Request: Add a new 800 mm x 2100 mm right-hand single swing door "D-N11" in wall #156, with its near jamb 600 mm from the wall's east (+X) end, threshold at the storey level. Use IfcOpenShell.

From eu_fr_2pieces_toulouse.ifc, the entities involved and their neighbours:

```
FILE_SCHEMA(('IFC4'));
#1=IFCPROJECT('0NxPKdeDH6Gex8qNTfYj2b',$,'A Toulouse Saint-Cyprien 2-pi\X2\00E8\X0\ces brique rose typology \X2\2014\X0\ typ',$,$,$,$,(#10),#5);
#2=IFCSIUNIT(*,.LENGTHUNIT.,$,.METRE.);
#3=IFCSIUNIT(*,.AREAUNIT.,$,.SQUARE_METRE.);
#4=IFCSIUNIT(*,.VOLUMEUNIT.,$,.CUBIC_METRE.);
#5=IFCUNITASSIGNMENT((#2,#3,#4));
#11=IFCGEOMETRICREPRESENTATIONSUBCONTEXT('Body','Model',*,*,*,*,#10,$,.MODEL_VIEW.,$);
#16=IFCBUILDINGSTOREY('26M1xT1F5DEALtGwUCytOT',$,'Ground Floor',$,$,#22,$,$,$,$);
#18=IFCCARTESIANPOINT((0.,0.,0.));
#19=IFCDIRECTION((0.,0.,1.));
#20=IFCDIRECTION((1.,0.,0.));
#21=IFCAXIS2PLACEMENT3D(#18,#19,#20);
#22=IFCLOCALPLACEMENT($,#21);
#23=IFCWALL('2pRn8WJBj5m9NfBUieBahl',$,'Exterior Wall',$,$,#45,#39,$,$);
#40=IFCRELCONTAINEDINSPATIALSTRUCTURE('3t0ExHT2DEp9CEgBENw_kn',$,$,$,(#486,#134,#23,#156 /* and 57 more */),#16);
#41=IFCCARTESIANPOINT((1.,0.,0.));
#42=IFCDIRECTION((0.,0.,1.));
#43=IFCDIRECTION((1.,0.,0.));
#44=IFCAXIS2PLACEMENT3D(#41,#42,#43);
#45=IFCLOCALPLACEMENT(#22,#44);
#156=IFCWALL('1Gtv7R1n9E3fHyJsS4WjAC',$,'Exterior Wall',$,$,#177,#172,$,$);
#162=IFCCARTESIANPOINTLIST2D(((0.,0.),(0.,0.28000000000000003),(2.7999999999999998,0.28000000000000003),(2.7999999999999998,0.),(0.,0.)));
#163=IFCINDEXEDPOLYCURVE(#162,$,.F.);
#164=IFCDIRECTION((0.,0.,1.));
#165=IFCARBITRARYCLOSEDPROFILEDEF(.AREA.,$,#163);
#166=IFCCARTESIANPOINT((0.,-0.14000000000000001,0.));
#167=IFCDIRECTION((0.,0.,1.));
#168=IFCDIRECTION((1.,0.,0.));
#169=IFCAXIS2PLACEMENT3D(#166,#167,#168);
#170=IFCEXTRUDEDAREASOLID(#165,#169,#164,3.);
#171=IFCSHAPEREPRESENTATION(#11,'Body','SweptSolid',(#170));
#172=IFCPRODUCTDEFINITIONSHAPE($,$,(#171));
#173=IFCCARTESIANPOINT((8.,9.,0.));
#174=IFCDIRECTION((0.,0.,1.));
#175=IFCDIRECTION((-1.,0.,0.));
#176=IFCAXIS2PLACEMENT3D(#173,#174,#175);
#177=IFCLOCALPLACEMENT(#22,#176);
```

```python
import numpy as np
import ifcopenshell
import ifcopenshell.api.feature
import ifcopenshell.api.geometry
import ifcopenshell.api.root
import ifcopenshell.api.spatial
import ifcopenshell.geom
import ifcopenshell.util.element
import ifcopenshell.util.placement
import ifcopenshell.util.representation
import ifcopenshell.util.shape
import ifcopenshell.util.unit

model = ifcopenshell.open("eu_fr_2pieces_toulouse.ifc")
unit_scale = ifcopenshell.util.unit.calculate_unit_scale(model)
settings = ifcopenshell.geom.settings()


def volume(element):
    """Net volume in cubic metres, openings subtracted."""
    shape = ifcopenshell.geom.create_shape(settings, element)
    return ifcopenshell.util.shape.get_volume(shape.geometry)


wall = model.by_id(156)
storey = ifcopenshell.util.element.get_container(wall, ifc_class="IfcBuildingStorey")
context = ifcopenshell.util.representation.get_context(model, "Model", "Body", "MODEL_VIEW")
before = volume(wall)

width, height, from_end, sill = 0.8, 2.1, 0.6, 0.0  # metres

# The wall runs along its own X axis, and the end named is its -X end.
wall_shape = ifcopenshell.geom.create_shape(settings, wall)
x, y, z = ifcopenshell.util.shape.get_vertices(wall_shape.geometry).T
start = x.min() + from_end
face, thickness = float(y.min()), float(y.max() - y.min())
wall_matrix = ifcopenshell.util.placement.get_local_placement(wall.ObjectPlacement)
level = ifcopenshell.util.placement.get_local_placement(storey.ObjectPlacement)[2, 3]


def in_wall(x, y):
    """Placement at x, y metres in the wall's axes, at sill height."""
    matrix = wall_matrix.copy()
    matrix[:, 3] = wall_matrix @ np.array([x / unit_scale, y / unit_scale, 0.0, 1.0])
    matrix[2, 3] = level + sill / unit_scale
    return matrix


# Opening: a box that overshoots both wall faces by 50 mm.
opening = ifcopenshell.api.root.create_entity(model, ifc_class="IfcOpeningElement", predefined_type="OPENING")
box = ifcopenshell.api.geometry.add_wall_representation(
    model, context=context, length=width, height=height, thickness=thickness + 0.1
)
ifcopenshell.api.geometry.assign_representation(model, product=opening, representation=box)
ifcopenshell.api.geometry.edit_object_placement(model, product=opening, matrix=in_wall(start, face - 0.05), is_si=False)
ifcopenshell.api.feature.add_feature(model, feature=opening, element=wall)

door = ifcopenshell.api.root.create_entity(model, ifc_class="IfcDoor", name="D-N11", predefined_type="DOOR")
door.OverallWidth, door.OverallHeight = width / unit_scale, height / unit_scale
door.OperationType = "SINGLE_SWING_RIGHT"
body = ifcopenshell.api.geometry.add_door_representation(
    model,
    context=context,
    overall_width=door.OverallWidth,
    overall_height=door.OverallHeight,
    operation_type="SINGLE_SWING_RIGHT",
    lining_properties={"LiningDepth": thickness / unit_scale, "ThresholdDepth": thickness / unit_scale},
)
ifcopenshell.api.geometry.assign_representation(model, product=door, representation=body)
ifcopenshell.api.spatial.assign_container(model, products=[door], relating_structure=storey)
ifcopenshell.api.feature.add_filling(model, opening=opening, element=door)

# The lining spans the wall, so the door starts at the wall face.
ifcopenshell.api.geometry.edit_object_placement(model, product=door, matrix=in_wall(start, face), is_si=False)

after = volume(wall)

print(f"wall volume {before:.3f} -> {after:.3f} m3")

model.write("eu_fr_2pieces_toulouse_edited.ifc")
```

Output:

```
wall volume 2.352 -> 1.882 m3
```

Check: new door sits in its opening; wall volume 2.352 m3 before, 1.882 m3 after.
